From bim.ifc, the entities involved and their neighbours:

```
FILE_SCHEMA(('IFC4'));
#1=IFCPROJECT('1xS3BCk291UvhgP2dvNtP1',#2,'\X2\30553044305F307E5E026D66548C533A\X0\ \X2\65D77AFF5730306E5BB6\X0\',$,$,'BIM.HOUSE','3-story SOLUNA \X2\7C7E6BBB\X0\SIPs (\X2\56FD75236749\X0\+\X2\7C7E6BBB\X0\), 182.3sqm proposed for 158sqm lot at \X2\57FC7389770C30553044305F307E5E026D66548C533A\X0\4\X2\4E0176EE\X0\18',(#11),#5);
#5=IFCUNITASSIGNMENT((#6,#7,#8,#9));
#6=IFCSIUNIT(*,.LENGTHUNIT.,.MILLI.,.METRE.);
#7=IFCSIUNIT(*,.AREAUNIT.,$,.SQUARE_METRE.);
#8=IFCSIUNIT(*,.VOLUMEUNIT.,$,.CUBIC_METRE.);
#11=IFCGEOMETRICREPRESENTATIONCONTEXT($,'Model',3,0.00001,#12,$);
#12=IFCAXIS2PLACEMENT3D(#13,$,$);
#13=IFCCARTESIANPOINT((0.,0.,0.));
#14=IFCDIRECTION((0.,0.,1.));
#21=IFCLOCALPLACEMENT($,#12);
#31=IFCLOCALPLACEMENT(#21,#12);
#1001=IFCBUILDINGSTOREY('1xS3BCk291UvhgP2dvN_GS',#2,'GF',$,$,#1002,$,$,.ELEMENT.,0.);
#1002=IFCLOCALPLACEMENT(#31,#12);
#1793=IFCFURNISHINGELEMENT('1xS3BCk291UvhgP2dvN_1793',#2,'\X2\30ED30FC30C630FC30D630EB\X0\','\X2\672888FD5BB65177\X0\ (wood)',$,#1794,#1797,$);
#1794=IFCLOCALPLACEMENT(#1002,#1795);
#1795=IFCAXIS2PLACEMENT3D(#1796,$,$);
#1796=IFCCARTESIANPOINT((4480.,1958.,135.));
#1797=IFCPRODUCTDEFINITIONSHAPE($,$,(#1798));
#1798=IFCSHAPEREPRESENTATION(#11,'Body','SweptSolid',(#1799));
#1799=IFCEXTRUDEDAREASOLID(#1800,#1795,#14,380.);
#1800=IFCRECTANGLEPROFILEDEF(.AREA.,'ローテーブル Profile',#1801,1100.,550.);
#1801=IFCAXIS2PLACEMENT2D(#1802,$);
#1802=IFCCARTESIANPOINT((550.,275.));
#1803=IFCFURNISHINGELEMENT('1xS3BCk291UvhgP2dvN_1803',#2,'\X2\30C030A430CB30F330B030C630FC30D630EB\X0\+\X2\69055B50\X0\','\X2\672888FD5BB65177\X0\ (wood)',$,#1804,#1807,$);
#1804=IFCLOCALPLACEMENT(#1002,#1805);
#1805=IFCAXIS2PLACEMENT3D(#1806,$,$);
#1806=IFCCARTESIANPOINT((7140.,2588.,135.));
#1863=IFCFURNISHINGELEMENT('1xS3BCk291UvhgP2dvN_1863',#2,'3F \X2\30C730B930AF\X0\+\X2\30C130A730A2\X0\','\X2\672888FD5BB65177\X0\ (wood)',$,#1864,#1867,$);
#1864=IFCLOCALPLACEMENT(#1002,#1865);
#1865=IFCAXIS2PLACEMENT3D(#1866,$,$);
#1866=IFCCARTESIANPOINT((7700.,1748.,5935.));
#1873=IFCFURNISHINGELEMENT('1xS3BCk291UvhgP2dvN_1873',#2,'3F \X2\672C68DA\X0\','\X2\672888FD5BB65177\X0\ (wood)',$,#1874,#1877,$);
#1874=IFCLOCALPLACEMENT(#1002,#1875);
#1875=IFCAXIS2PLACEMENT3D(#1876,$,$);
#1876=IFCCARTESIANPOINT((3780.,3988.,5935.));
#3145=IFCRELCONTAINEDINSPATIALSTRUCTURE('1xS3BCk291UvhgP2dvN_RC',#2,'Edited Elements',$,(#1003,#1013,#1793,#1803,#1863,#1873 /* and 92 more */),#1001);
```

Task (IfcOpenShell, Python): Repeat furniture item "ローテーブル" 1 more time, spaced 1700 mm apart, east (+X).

```python
import numpy as np
import ifcopenshell
import ifcopenshell.api.geometry
import ifcopenshell.api.root
import ifcopenshell.util.element
import ifcopenshell.util.placement

model = ifcopenshell.open("bim.ifc")


def reuse_history(source, copy):
    """copy_class also copies each property set's owner history, people and application; keep the originals."""
    for rel in copy.IsDefinedBy:
        if rel.is_a("IfcRelDefinesByProperties") and (history := rel.RelatingPropertyDefinition.OwnerHistory):
            rel.RelatingPropertyDefinition.OwnerHistory = source.OwnerHistory
            ifcopenshell.util.element.remove_deep2(model, history)


source = model.by_id(1793)
base = ifcopenshell.util.placement.get_local_placement(source.ObjectPlacement)
step = np.array([1.0, 0.0, 0.0]) * 1700.0

for i in range(1, 2):
    copy = ifcopenshell.api.root.copy_class(model, product=source)
    copy.Representation = ifcopenshell.util.element.copy_deep(
        model, source.Representation, exclude=["IfcGeometricRepresentationContext", "IfcRepresentationMap"]
    )
    reuse_history(source, copy)
    matrix = base.copy()
    matrix[:3, 3] += i * step
    print("added at", matrix[:3, 3].round(3) + 0.0)
    ifcopenshell.api.geometry.edit_object_placement(model, product=copy, matrix=matrix, is_si=False)

model.write("bim_updated.ifc")
```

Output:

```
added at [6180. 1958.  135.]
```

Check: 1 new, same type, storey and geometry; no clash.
